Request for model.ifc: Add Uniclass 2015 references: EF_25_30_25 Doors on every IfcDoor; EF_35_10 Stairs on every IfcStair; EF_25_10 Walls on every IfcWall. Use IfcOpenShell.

First a look at what the model holds.

```python
import ifcopenshell

model = ifcopenshell.open("model.ifc")
print(model.schema)
print("classifications:", [c.Name for c in model.by_type("IfcClassification")])
for ifc_class in ("IfcDoor", "IfcRoof", "IfcStair", "IfcWall", "IfcWindow"):
    print(ifc_class, len(model.by_type(ifc_class)))
```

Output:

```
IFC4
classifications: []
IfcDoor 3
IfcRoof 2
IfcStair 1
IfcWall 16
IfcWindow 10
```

```python
import ifcopenshell
import ifcopenshell.api.classification

model = ifcopenshell.open("model.ifc")

system = ifcopenshell.api.classification.add_classification(model, classification="Uniclass 2015")

codes = {
    "IfcDoor": ("EF_25_30_25", "Doors"),
    "IfcStair": ("EF_35_10", "Stairs"),
    "IfcWall": ("EF_25_10", "Walls"),
}
for ifc_class, (code, name) in codes.items():
    products = model.by_type(ifc_class)
    ifcopenshell.api.classification.add_reference(
        model, products=products, classification=system, identification=code, name=name
    )
    print(code, len(products))

model.write("model_v2.ifc")
```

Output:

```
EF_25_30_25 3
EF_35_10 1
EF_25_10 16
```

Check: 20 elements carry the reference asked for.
